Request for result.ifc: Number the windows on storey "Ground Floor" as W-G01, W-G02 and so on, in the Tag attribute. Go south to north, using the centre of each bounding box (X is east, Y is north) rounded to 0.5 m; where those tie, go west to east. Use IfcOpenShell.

First a look at what the model holds.

```python
import ifcopenshell
import ifcopenshell.util.element
import ifcopenshell.util.placement

model = ifcopenshell.open("result.ifc")
print(model.schema)
storey = next(s for s in model.by_type("IfcBuildingStorey") if s.Name == "Ground Floor")
windows = [e for e in ifcopenshell.util.element.get_decomposition(storey) if e.is_a("IfcWindow")]
for e in sorted(windows, key=lambda e: e.id()):
    origin = ifcopenshell.util.placement.get_local_placement(e.ObjectPlacement)[:3, 3]
    print(e.id(), e.Tag, e.Name, origin.round(2) + 0.0, sep=" | ")
```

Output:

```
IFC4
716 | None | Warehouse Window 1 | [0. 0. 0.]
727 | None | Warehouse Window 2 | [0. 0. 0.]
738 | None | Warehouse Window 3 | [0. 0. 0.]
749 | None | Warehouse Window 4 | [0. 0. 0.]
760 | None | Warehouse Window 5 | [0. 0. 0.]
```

```python
import ifcopenshell
import ifcopenshell.geom
import ifcopenshell.util.element
import ifcopenshell.util.shape

model = ifcopenshell.open("result.ifc")
settings = ifcopenshell.geom.settings()
settings.set("use-world-coords", True)


def centre(element):
    shape = ifcopenshell.geom.create_shape(settings, element)
    return ifcopenshell.util.shape.get_bbox_centroid(shape.geometry)


storey = next(s for s in model.by_type("IfcBuildingStorey") if s.Name == "Ground Floor")
windows = [e for e in ifcopenshell.util.element.get_decomposition(storey) if e.is_a("IfcWindow")]

# Insertion points can sit at a corner or the storey origin, so sort by the geometry (in metres).
centres = {e: centre(e) for e in windows}
windows.sort(key=lambda e: (round(centres[e][1] / 0.5), centres[e][0]))

for i, e in enumerate(windows, start=1):
    number = f"W-G{i:02d}"
    e.Tag = number
    print(e.id(), number)

model.write("result_v2.ifc")
```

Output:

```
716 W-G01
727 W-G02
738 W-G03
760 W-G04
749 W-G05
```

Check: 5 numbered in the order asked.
